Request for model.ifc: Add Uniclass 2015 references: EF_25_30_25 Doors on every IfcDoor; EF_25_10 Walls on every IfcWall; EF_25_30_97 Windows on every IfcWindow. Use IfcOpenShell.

First a look at what the model holds.

```python
import ifcopenshell

model = ifcopenshell.open("model.ifc")
print(model.schema)
print("classifications:", [c.Name for c in model.by_type("IfcClassification")])
for ifc_class in ("IfcDoor", "IfcRoof", "IfcStair", "IfcWall", "IfcWindow"):
    print(ifc_class, len(model.by_type(ifc_class)))
```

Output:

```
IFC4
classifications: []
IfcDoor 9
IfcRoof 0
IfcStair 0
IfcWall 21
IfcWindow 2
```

```python
import ifcopenshell
import ifcopenshell.api.classification

model = ifcopenshell.open("model.ifc")

system = ifcopenshell.api.classification.add_classification(model, classification="Uniclass 2015")

codes = {
    "IfcDoor": ("EF_25_30_25", "Doors"),
    "IfcWall": ("EF_25_10", "Walls"),
    "IfcWindow": ("EF_25_30_97", "Windows"),
}
for ifc_class, (code, name) in codes.items():
    products = model.by_type(ifc_class)
    ifcopenshell.api.classification.add_reference(
        model, products=products, classification=system, identification=code, name=name
    )
    print(code, len(products))

model.write("model_updated.ifc")
```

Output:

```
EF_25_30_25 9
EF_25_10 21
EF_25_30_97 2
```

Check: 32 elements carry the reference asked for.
